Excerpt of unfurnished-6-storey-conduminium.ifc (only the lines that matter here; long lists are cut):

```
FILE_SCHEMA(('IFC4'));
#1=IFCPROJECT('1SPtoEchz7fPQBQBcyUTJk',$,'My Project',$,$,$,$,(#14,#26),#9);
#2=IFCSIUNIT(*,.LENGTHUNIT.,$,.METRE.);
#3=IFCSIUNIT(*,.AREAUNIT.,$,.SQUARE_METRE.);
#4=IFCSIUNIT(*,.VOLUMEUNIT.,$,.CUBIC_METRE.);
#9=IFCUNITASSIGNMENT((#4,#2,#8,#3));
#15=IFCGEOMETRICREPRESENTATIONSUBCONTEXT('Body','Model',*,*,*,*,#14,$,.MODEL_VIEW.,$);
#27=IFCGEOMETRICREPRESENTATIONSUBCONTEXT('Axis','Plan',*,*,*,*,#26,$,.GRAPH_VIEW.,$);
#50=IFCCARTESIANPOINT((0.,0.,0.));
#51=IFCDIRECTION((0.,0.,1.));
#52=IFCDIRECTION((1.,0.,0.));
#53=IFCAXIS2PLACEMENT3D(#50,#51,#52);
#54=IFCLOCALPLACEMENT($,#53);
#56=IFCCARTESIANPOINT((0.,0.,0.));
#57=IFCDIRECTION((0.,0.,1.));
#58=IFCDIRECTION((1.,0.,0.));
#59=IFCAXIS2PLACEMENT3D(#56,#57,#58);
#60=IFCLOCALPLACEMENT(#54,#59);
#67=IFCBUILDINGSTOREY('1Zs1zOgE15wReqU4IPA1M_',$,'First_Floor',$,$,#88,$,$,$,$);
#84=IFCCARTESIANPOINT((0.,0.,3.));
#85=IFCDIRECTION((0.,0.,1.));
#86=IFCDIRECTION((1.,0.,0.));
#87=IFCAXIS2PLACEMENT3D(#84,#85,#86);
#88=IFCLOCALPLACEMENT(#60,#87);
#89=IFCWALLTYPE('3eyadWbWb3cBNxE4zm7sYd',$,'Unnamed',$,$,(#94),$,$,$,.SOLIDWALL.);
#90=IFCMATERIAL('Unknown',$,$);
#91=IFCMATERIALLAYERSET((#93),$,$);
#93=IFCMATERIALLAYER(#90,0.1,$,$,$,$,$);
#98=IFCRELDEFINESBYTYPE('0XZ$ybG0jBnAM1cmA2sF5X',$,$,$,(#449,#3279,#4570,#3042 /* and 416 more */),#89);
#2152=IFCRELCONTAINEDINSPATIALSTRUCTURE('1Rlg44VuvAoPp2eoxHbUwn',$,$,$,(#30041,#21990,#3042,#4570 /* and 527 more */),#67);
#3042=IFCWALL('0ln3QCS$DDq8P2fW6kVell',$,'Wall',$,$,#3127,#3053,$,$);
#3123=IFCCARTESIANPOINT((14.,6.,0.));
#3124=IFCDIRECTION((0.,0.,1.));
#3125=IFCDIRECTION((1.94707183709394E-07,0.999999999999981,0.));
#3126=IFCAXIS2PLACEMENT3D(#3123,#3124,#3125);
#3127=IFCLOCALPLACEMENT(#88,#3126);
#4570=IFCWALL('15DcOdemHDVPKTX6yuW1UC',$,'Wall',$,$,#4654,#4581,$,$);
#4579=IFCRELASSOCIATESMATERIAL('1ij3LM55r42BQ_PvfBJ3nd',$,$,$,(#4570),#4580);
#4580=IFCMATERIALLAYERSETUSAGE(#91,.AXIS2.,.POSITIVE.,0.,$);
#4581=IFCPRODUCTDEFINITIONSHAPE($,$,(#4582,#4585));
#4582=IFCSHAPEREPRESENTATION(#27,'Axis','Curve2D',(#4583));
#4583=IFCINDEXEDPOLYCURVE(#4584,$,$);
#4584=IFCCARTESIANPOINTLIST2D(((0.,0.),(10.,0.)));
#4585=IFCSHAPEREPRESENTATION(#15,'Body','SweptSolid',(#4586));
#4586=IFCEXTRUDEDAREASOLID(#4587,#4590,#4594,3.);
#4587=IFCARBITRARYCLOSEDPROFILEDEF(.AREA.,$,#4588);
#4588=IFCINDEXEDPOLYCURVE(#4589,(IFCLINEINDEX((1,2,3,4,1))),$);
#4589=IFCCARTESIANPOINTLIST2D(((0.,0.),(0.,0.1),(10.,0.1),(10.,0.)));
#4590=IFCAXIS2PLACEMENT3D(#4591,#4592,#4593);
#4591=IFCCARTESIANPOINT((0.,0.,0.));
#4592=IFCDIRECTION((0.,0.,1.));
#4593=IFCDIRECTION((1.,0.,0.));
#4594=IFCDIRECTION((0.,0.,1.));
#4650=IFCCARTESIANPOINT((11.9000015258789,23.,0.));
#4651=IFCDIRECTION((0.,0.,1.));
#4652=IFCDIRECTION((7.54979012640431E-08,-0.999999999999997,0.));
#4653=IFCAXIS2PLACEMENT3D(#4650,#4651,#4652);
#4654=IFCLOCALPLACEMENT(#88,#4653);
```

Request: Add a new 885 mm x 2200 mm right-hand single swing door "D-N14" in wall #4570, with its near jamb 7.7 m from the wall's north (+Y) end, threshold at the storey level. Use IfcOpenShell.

```python
import numpy as np
import ifcopenshell
import ifcopenshell.api.feature
import ifcopenshell.api.geometry
import ifcopenshell.api.root
import ifcopenshell.api.spatial
import ifcopenshell.geom
import ifcopenshell.util.element
import ifcopenshell.util.placement
import ifcopenshell.util.representation
import ifcopenshell.util.shape
import ifcopenshell.util.unit

model = ifcopenshell.open("unfurnished-6-storey-conduminium.ifc")
unit_scale = ifcopenshell.util.unit.calculate_unit_scale(model)
settings = ifcopenshell.geom.settings()


def volume(element):
    """Net volume in cubic metres, openings subtracted."""
    shape = ifcopenshell.geom.create_shape(settings, element)
    return ifcopenshell.util.shape.get_volume(shape.geometry)


wall = model.by_guid("15DcOdemHDVPKTX6yuW1UC")
storey = ifcopenshell.util.element.get_container(wall, ifc_class="IfcBuildingStorey")
context = ifcopenshell.util.representation.get_context(model, "Model", "Body", "MODEL_VIEW")
before = volume(wall)

width, height, from_end, sill = 0.885, 2.2, 7.7, 0.0  # metres

# The wall runs along its own X axis, and the end named is its -X end.
wall_shape = ifcopenshell.geom.create_shape(settings, wall)
x, y, z = ifcopenshell.util.shape.get_vertices(wall_shape.geometry).T
start = x.min() + from_end
face, thickness = float(y.min()), float(y.max() - y.min())
wall_matrix = ifcopenshell.util.placement.get_local_placement(wall.ObjectPlacement)
level = ifcopenshell.util.placement.get_local_placement(storey.ObjectPlacement)[2, 3]


def in_wall(x, y):
    """Placement at x, y metres in the wall's axes, at sill height."""
    matrix = wall_matrix.copy()
    matrix[:, 3] = wall_matrix @ np.array([x / unit_scale, y / unit_scale, 0.0, 1.0])
    matrix[2, 3] = level + sill / unit_scale
    return matrix


# Opening: a box that overshoots both wall faces by 50 mm.
opening = ifcopenshell.api.root.create_entity(model, ifc_class="IfcOpeningElement", predefined_type="OPENING")
box = ifcopenshell.api.geometry.add_wall_representation(
    model, context=context, length=width, height=height, thickness=thickness + 0.1
)
ifcopenshell.api.geometry.assign_representation(model, product=opening, representation=box)
ifcopenshell.api.geometry.edit_object_placement(model, product=opening, matrix=in_wall(start, face - 0.05), is_si=False)
ifcopenshell.api.feature.add_feature(model, feature=opening, element=wall)

door = ifcopenshell.api.root.create_entity(model, ifc_class="IfcDoor", name="D-N14", predefined_type="DOOR")
door.OverallWidth, door.OverallHeight = width / unit_scale, height / unit_scale
door.OperationType = "SINGLE_SWING_RIGHT"
body = ifcopenshell.api.geometry.add_door_representation(
    model,
    context=context,
    overall_width=door.OverallWidth,
    overall_height=door.OverallHeight,
    operation_type="SINGLE_SWING_RIGHT",
    lining_properties={"LiningDepth": thickness / unit_scale, "ThresholdDepth": thickness / unit_scale},
)
ifcopenshell.api.geometry.assign_representation(model, product=door, representation=body)
ifcopenshell.api.spatial.assign_container(model, products=[door], relating_structure=storey)
ifcopenshell.api.feature.add_filling(model, opening=opening, element=door)

# The lining spans the wall, so the door starts at the wall face.
ifcopenshell.api.geometry.edit_object_placement(model, product=door, matrix=in_wall(start, face), is_si=False)

after = volume(wall)

print(f"wall volume {before:.3f} -> {after:.3f} m3")

model.write("unfurnished-6-storey-conduminium_v2.ifc")
```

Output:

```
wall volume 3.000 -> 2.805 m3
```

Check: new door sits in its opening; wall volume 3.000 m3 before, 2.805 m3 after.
